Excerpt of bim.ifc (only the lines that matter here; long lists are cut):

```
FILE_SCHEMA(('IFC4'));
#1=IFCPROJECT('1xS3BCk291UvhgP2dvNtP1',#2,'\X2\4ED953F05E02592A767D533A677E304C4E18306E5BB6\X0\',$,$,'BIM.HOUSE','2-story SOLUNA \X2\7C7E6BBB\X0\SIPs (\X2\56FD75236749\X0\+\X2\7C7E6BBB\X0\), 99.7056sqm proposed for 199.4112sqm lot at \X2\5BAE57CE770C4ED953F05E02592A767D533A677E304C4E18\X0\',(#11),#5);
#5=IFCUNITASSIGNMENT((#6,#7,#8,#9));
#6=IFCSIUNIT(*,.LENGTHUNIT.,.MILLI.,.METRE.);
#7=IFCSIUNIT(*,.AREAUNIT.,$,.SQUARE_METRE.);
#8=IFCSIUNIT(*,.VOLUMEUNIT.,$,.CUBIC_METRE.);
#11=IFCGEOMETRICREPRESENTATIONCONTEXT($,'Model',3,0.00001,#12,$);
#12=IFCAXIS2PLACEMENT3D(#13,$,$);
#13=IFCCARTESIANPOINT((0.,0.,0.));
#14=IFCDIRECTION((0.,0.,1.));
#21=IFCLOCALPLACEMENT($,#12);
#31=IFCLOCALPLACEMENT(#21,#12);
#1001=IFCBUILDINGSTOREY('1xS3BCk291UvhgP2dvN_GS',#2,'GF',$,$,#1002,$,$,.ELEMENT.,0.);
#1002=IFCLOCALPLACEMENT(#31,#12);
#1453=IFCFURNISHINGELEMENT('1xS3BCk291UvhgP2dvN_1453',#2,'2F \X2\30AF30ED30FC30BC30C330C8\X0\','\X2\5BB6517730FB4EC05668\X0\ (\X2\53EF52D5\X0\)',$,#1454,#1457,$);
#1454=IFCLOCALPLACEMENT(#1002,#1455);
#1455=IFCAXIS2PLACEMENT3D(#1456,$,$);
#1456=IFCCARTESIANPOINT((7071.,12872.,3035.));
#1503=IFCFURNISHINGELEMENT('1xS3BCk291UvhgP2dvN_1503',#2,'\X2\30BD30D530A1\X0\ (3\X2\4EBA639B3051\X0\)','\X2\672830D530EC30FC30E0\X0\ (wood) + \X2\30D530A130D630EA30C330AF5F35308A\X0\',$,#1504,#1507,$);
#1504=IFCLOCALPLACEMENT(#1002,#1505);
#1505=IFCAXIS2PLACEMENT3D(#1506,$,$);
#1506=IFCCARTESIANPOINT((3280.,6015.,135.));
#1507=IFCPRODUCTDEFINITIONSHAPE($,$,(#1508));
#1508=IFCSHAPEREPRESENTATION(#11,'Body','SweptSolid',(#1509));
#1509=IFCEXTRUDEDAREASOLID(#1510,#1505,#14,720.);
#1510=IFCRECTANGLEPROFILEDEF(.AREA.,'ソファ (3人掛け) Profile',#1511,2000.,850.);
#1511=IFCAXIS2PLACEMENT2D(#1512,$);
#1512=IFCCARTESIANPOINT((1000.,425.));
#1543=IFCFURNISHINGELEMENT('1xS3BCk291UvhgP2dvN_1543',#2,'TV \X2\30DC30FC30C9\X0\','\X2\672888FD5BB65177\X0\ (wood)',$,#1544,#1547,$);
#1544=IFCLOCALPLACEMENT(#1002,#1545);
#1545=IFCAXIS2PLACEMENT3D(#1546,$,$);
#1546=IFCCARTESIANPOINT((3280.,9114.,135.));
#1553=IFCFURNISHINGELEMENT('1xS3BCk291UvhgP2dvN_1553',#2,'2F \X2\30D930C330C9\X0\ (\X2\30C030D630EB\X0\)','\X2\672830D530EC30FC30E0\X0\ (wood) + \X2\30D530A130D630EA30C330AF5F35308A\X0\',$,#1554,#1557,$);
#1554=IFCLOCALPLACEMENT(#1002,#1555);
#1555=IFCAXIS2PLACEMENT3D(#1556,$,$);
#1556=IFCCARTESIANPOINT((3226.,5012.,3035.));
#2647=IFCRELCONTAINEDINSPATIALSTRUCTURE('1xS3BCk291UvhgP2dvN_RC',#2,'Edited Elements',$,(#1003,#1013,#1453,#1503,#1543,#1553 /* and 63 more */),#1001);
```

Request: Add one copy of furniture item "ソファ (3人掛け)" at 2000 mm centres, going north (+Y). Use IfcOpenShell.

```python
import numpy as np
import ifcopenshell
import ifcopenshell.api.geometry
import ifcopenshell.api.root
import ifcopenshell.util.element
import ifcopenshell.util.placement
import ifcopenshell.util.unit

model = ifcopenshell.open("bim.ifc")
unit_scale = ifcopenshell.util.unit.calculate_unit_scale(model)


def reuse_history(source, copy):
    """copy_class also copies each property set's owner history, people and application; keep the originals."""
    for rel in copy.IsDefinedBy:
        if rel.is_a("IfcRelDefinesByProperties") and (history := rel.RelatingPropertyDefinition.OwnerHistory):
            rel.RelatingPropertyDefinition.OwnerHistory = source.OwnerHistory
            ifcopenshell.util.element.remove_deep2(model, history)


source = model.by_guid("1xS3BCk291UvhgP2dvN_1503")
base = ifcopenshell.util.placement.get_local_placement(source.ObjectPlacement)
step = np.array([0.0, 1.0, 0.0]) * 2 / unit_scale

for i in range(1, 2):
    copy = ifcopenshell.api.root.copy_class(model, product=source)
    copy.Representation = ifcopenshell.util.element.copy_deep(
        model, source.Representation, exclude=["IfcGeometricRepresentationContext", "IfcRepresentationMap"]
    )
    reuse_history(source, copy)
    matrix = base.copy()
    matrix[:3, 3] += i * step
    print("added at", matrix[:3, 3].round(3) + 0.0)
    ifcopenshell.api.geometry.edit_object_placement(model, product=copy, matrix=matrix, is_si=False)

model.write("bim_rev.ifc")
```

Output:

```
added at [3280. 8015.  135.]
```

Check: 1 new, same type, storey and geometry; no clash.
